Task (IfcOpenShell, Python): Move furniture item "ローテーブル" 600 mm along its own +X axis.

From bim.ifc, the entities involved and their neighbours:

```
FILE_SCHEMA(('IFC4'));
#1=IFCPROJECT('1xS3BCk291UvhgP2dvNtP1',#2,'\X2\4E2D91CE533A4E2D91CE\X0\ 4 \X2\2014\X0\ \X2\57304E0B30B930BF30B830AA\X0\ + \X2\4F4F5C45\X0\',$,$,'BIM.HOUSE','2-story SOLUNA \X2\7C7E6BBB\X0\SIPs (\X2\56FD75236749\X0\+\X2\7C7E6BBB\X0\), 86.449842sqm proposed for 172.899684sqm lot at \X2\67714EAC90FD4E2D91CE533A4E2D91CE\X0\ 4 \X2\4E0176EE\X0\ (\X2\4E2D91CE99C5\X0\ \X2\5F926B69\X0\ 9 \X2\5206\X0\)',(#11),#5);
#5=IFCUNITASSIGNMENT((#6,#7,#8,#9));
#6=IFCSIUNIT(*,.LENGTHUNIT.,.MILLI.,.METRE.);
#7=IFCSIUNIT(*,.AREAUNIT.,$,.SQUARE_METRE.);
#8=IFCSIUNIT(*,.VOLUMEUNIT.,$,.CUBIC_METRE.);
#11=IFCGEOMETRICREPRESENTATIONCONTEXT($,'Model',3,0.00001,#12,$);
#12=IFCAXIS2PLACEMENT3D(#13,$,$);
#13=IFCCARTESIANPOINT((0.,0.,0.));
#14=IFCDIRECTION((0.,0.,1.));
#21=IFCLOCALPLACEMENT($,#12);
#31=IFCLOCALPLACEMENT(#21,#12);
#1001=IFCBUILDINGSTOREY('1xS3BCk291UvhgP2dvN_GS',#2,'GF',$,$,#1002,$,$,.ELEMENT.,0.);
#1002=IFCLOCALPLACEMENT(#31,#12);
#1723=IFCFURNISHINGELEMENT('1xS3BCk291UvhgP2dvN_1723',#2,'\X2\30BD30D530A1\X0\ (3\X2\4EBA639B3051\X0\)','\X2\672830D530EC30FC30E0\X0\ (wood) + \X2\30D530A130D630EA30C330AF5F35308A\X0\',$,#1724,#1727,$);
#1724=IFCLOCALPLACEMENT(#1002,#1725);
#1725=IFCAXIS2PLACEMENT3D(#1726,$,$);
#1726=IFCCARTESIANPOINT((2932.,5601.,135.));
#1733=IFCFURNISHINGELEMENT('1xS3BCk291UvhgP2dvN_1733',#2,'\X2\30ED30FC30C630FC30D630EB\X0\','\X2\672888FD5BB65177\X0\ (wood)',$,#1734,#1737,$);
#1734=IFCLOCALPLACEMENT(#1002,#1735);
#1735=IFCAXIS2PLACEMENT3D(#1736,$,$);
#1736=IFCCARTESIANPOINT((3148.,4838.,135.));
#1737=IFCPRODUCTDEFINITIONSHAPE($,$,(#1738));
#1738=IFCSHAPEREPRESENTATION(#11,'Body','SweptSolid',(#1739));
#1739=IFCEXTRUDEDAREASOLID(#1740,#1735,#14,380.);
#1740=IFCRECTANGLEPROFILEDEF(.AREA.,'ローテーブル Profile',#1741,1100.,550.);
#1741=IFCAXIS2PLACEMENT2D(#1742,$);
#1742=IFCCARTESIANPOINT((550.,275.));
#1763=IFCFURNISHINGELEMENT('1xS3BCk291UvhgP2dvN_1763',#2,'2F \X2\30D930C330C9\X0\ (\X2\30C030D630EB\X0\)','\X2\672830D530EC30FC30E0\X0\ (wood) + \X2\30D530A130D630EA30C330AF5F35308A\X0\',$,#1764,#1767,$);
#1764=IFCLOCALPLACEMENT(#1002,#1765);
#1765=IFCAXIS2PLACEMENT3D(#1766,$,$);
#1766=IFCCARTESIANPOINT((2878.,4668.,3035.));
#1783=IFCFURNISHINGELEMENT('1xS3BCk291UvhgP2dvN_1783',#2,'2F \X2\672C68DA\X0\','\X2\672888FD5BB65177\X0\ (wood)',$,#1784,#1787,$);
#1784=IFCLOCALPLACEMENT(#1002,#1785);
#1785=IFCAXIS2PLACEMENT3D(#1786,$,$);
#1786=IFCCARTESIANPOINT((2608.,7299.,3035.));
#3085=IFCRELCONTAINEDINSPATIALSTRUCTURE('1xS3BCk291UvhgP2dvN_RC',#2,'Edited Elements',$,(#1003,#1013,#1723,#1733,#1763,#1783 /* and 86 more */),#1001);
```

```python
import ifcopenshell
import ifcopenshell.api.geometry
import ifcopenshell.util.placement
import ifcopenshell.util.unit

model = ifcopenshell.open("bim.ifc")
unit_scale = ifcopenshell.util.unit.calculate_unit_scale(model)

item = model.by_guid("1xS3BCk291UvhgP2dvN_1733")
matrix = ifcopenshell.util.placement.get_local_placement(item.ObjectPlacement)
matrix[:3, 3] += matrix[:3, 0] * 0.6 / unit_scale
ifcopenshell.api.geometry.edit_object_placement(model, product=item, matrix=matrix, is_si=False)

print(ifcopenshell.util.placement.get_local_placement(item.ObjectPlacement).round(3) + 0.0)

model.write("bim_rev.ifc")
```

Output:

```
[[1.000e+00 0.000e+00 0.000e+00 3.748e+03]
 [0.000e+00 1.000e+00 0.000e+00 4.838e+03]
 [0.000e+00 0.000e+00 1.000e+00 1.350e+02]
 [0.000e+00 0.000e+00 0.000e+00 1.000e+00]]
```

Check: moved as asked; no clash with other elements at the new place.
